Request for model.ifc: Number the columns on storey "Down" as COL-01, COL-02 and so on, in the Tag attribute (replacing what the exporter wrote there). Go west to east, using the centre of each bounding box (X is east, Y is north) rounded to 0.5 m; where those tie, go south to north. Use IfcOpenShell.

First a look at what the model holds.

```python
import ifcopenshell
import ifcopenshell.util.element
import ifcopenshell.util.placement

model = ifcopenshell.open("model.ifc")
print(model.schema)
storey = next(s for s in model.by_type("IfcBuildingStorey") if s.Name == "Down")
columns = [e for e in ifcopenshell.util.element.get_decomposition(storey) if e.is_a("IfcColumn")]
for e in sorted(columns, key=lambda e: e.id()):
    origin = ifcopenshell.util.placement.get_local_placement(e.ObjectPlacement)[:3, 3]
    print(e.id(), e.Tag, e.Name, origin.round(2) + 0.0, sep=" | ")
```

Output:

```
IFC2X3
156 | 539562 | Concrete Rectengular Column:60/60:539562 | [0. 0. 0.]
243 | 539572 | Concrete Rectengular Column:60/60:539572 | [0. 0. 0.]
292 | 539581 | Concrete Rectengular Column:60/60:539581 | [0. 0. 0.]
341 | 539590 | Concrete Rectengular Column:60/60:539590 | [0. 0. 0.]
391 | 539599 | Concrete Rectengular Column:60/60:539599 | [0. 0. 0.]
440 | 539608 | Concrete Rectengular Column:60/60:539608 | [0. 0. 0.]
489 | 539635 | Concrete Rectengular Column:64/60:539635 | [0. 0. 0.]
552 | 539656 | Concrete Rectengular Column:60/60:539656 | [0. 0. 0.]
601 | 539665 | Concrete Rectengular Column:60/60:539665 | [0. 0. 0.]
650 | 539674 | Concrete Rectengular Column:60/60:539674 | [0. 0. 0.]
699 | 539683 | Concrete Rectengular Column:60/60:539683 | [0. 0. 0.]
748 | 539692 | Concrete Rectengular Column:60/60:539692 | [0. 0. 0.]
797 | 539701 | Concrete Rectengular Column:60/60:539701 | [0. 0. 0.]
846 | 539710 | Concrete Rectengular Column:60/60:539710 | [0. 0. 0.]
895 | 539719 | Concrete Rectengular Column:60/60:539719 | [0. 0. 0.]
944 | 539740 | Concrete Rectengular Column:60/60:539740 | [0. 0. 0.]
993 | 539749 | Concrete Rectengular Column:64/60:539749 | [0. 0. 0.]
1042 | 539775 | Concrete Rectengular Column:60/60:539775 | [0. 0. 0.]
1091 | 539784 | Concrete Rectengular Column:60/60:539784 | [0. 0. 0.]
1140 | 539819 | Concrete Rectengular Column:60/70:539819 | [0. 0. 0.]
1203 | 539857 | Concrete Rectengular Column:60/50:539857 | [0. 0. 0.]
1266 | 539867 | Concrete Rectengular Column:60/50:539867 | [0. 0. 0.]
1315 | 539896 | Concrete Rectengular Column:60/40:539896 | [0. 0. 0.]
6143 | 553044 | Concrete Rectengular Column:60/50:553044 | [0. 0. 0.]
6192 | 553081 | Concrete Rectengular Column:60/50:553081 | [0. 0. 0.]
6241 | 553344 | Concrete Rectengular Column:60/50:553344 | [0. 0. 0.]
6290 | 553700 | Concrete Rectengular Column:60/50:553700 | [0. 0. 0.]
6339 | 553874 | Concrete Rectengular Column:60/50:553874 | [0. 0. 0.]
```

```python
import ifcopenshell
import ifcopenshell.geom
import ifcopenshell.util.element
import ifcopenshell.util.shape

model = ifcopenshell.open("model.ifc")
settings = ifcopenshell.geom.settings()
settings.set("use-world-coords", True)


def centre(element):
    shape = ifcopenshell.geom.create_shape(settings, element)
    return ifcopenshell.util.shape.get_bbox_centroid(shape.geometry)


storey = next(s for s in model.by_type("IfcBuildingStorey") if s.Name == "Down")
columns = [e for e in ifcopenshell.util.element.get_decomposition(storey) if e.is_a("IfcColumn")]

# Insertion points can sit at a corner or the storey origin, so sort by the geometry (in metres).
centres = {e: centre(e) for e in columns}
columns.sort(key=lambda e: (round(centres[e][0] / 0.5), centres[e][1]))

for i, e in enumerate(columns, start=1):
    number = f"COL-{i:02d}"
    e.Tag = number
    print(e.id(), number)

model.write("model_updated.ifc")
```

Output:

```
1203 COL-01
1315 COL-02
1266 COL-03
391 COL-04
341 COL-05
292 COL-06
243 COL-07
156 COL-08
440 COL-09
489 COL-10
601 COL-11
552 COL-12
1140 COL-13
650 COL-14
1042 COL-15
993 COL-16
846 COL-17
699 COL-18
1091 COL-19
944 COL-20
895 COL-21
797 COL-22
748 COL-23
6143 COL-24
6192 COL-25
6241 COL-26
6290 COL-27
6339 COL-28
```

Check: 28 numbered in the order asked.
